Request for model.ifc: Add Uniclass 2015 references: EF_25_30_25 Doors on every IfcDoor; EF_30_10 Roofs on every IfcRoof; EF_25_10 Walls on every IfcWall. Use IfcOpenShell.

First a look at what the model holds.

```python
import ifcopenshell

model = ifcopenshell.open("model.ifc")
print(model.schema)
print("classifications:", [c.Name for c in model.by_type("IfcClassification")])
for ifc_class in ("IfcDoor", "IfcRoof", "IfcStair", "IfcWall", "IfcWindow"):
    print(ifc_class, len(model.by_type(ifc_class)))
```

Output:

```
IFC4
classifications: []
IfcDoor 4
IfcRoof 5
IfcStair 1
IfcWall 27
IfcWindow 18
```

```python
import ifcopenshell
import ifcopenshell.api.classification

model = ifcopenshell.open("model.ifc")

system = ifcopenshell.api.classification.add_classification(model, classification="Uniclass 2015")

codes = {
    "IfcDoor": ("EF_25_30_25", "Doors"),
    "IfcRoof": ("EF_30_10", "Roofs"),
    "IfcWall": ("EF_25_10", "Walls"),
}
for ifc_class, (code, name) in codes.items():
    products = model.by_type(ifc_class)
    ifcopenshell.api.classification.add_reference(
        model, products=products, classification=system, identification=code, name=name
    )
    print(code, len(products))

model.write("model_edited.ifc")
```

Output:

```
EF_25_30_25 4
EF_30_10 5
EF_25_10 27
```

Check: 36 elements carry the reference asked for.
